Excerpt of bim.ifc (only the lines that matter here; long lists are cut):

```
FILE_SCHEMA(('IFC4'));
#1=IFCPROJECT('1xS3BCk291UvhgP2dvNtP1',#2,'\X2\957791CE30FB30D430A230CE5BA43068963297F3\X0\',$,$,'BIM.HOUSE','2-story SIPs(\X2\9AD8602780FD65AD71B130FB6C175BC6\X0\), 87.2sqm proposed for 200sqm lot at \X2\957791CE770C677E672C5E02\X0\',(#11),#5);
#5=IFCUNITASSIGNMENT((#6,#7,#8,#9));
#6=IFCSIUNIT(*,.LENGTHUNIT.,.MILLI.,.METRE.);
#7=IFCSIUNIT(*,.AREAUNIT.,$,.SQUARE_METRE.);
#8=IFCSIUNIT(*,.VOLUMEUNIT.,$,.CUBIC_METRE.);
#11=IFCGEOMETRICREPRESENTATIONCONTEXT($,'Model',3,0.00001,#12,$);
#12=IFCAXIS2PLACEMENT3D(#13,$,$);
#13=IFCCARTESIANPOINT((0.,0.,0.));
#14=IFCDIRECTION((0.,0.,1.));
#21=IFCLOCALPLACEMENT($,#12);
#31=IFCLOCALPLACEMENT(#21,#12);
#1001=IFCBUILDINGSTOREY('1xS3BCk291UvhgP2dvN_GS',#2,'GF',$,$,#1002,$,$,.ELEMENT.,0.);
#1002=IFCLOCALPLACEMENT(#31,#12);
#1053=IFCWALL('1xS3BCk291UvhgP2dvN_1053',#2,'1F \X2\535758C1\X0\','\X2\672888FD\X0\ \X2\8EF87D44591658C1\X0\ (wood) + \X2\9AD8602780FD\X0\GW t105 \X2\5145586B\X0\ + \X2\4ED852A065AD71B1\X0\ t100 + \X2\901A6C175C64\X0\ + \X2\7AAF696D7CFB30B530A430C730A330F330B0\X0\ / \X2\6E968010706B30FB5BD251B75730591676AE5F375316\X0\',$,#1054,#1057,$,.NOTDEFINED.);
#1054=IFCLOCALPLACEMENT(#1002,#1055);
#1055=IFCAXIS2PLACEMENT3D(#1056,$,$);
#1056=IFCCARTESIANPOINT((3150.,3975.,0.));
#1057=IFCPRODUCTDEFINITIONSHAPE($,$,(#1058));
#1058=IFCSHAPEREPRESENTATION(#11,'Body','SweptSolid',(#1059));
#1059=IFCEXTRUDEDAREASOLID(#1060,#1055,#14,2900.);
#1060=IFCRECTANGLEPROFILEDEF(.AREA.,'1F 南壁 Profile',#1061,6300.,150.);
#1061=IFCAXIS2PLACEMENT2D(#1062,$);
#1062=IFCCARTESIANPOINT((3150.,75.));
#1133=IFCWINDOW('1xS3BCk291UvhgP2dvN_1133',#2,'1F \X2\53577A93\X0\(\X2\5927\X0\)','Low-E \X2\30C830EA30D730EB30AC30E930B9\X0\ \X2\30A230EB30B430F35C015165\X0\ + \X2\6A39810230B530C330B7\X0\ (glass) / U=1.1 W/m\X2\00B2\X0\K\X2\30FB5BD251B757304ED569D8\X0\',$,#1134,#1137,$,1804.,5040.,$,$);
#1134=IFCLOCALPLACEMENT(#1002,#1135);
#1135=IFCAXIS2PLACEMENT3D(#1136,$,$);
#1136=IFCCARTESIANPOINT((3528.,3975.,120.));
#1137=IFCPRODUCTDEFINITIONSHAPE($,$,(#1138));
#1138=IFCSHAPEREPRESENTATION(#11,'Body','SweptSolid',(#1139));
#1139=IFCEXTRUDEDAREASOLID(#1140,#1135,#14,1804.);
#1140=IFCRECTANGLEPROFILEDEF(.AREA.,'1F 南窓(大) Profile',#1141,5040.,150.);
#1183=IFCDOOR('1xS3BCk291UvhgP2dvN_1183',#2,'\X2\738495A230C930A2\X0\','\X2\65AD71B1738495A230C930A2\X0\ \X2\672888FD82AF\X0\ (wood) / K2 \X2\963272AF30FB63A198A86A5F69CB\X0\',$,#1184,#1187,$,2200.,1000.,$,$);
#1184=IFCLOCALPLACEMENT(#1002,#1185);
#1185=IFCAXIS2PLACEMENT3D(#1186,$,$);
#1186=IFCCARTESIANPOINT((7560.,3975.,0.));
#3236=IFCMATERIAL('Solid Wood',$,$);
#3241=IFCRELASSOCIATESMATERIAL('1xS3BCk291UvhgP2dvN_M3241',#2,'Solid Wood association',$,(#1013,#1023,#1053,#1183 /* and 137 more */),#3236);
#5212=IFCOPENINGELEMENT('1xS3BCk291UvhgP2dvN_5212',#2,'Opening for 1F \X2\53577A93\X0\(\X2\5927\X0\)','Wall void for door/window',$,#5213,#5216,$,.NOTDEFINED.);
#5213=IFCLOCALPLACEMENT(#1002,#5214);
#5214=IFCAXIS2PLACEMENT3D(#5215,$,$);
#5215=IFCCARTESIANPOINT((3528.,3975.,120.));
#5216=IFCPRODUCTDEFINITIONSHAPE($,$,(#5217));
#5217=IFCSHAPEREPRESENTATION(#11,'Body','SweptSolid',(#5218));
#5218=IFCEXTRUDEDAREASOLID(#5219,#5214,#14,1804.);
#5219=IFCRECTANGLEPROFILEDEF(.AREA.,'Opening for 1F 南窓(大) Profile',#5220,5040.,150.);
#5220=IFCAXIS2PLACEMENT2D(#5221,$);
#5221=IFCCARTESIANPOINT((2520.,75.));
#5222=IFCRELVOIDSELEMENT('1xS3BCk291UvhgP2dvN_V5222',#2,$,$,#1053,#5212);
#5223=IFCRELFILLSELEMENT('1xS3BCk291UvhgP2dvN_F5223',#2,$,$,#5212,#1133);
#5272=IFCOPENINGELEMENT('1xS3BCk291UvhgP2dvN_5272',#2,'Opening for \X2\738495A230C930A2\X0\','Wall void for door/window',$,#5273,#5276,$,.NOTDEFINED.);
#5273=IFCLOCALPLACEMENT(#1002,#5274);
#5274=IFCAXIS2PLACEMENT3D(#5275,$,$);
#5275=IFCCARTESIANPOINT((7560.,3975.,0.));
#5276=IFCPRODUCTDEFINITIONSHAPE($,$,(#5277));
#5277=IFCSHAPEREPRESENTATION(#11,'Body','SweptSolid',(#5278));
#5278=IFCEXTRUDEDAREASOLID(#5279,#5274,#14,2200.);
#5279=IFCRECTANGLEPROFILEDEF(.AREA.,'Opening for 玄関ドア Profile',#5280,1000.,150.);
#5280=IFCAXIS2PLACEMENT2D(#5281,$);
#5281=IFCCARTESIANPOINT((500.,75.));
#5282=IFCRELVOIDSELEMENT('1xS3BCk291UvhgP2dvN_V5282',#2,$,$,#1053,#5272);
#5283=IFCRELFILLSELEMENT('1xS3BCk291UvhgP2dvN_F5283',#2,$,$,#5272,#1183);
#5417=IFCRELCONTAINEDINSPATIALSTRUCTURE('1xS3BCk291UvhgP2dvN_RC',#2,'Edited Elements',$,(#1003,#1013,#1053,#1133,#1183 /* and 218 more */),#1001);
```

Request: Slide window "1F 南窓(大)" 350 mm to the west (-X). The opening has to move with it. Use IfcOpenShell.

```python
import ifcopenshell
import ifcopenshell.api.geometry
import ifcopenshell.util.placement

model = ifcopenshell.open("bim.ifc")

window = model.by_guid("1xS3BCk291UvhgP2dvN_1133")
opening = window.FillsVoids[0].RelatingOpeningElement
wall = opening.VoidsElements[0].RelatingBuildingElement

wall_matrix = ifcopenshell.util.placement.get_local_placement(wall.ObjectPlacement)
shift = wall_matrix[:3, 0] * -350.0
before = ifcopenshell.util.placement.get_local_placement(window.ObjectPlacement)[:3, 3].copy()

# The window is not placed relative to its opening, so move both.
for product in (opening, window):
    matrix = ifcopenshell.util.placement.get_local_placement(product.ObjectPlacement)
    matrix[:3, 3] += shift
    ifcopenshell.api.geometry.edit_object_placement(model, product=product, matrix=matrix, is_si=False)

after = ifcopenshell.util.placement.get_local_placement(window.ObjectPlacement)[:3, 3]
print("window moved by", (after - before).round(3) + 0.0)

model.write("bim_rev.ifc")
```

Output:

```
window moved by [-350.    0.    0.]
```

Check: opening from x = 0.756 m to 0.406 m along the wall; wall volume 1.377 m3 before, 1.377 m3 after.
